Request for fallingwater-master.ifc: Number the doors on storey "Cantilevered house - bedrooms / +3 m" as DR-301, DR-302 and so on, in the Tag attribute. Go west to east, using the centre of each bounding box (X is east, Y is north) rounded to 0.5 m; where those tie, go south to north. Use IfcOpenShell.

First a look at what the model holds.

```python
import ifcopenshell
import ifcopenshell.util.element
import ifcopenshell.util.placement

model = ifcopenshell.open("fallingwater-master.ifc")
print(model.schema)
storey = next(s for s in model.by_type("IfcBuildingStorey") if s.Name == "Cantilevered house - bedrooms / +3 m")
doors = [e for e in ifcopenshell.util.element.get_decomposition(storey) if e.is_a("IfcDoor")]
for e in sorted(doors, key=lambda e: e.id()):
    origin = ifcopenshell.util.placement.get_local_placement(e.ObjectPlacement)[:3, 3]
    print(e.id(), e.Tag, e.Name, origin.round(2) + 0.0, sep=" | ")
```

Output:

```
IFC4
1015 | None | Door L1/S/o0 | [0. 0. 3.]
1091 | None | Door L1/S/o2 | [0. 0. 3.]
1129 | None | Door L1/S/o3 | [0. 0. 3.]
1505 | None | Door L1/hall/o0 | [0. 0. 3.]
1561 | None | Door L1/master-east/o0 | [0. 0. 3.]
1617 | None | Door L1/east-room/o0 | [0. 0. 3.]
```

```python
import ifcopenshell
import ifcopenshell.geom
import ifcopenshell.util.element
import ifcopenshell.util.shape

model = ifcopenshell.open("fallingwater-master.ifc")
settings = ifcopenshell.geom.settings()
settings.set("use-world-coords", True)


def centre(element):
    shape = ifcopenshell.geom.create_shape(settings, element)
    return ifcopenshell.util.shape.get_bbox_centroid(shape.geometry)


storey = next(s for s in model.by_type("IfcBuildingStorey") if s.Name == "Cantilevered house - bedrooms / +3 m")
doors = [e for e in ifcopenshell.util.element.get_decomposition(storey) if e.is_a("IfcDoor")]

# Insertion points can sit at a corner or the storey origin, so sort by the geometry (in metres).
centres = {e: centre(e) for e in doors}
doors.sort(key=lambda e: (round(centres[e][0] / 0.5), centres[e][1]))

for i, e in enumerate(doors, start=1):
    number = f"DR-3{i:02d}"
    e.Tag = number
    print(e.id(), number)

model.write("fallingwater-master-out.ifc")
```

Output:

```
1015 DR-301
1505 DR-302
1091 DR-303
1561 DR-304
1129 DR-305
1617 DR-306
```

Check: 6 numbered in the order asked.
